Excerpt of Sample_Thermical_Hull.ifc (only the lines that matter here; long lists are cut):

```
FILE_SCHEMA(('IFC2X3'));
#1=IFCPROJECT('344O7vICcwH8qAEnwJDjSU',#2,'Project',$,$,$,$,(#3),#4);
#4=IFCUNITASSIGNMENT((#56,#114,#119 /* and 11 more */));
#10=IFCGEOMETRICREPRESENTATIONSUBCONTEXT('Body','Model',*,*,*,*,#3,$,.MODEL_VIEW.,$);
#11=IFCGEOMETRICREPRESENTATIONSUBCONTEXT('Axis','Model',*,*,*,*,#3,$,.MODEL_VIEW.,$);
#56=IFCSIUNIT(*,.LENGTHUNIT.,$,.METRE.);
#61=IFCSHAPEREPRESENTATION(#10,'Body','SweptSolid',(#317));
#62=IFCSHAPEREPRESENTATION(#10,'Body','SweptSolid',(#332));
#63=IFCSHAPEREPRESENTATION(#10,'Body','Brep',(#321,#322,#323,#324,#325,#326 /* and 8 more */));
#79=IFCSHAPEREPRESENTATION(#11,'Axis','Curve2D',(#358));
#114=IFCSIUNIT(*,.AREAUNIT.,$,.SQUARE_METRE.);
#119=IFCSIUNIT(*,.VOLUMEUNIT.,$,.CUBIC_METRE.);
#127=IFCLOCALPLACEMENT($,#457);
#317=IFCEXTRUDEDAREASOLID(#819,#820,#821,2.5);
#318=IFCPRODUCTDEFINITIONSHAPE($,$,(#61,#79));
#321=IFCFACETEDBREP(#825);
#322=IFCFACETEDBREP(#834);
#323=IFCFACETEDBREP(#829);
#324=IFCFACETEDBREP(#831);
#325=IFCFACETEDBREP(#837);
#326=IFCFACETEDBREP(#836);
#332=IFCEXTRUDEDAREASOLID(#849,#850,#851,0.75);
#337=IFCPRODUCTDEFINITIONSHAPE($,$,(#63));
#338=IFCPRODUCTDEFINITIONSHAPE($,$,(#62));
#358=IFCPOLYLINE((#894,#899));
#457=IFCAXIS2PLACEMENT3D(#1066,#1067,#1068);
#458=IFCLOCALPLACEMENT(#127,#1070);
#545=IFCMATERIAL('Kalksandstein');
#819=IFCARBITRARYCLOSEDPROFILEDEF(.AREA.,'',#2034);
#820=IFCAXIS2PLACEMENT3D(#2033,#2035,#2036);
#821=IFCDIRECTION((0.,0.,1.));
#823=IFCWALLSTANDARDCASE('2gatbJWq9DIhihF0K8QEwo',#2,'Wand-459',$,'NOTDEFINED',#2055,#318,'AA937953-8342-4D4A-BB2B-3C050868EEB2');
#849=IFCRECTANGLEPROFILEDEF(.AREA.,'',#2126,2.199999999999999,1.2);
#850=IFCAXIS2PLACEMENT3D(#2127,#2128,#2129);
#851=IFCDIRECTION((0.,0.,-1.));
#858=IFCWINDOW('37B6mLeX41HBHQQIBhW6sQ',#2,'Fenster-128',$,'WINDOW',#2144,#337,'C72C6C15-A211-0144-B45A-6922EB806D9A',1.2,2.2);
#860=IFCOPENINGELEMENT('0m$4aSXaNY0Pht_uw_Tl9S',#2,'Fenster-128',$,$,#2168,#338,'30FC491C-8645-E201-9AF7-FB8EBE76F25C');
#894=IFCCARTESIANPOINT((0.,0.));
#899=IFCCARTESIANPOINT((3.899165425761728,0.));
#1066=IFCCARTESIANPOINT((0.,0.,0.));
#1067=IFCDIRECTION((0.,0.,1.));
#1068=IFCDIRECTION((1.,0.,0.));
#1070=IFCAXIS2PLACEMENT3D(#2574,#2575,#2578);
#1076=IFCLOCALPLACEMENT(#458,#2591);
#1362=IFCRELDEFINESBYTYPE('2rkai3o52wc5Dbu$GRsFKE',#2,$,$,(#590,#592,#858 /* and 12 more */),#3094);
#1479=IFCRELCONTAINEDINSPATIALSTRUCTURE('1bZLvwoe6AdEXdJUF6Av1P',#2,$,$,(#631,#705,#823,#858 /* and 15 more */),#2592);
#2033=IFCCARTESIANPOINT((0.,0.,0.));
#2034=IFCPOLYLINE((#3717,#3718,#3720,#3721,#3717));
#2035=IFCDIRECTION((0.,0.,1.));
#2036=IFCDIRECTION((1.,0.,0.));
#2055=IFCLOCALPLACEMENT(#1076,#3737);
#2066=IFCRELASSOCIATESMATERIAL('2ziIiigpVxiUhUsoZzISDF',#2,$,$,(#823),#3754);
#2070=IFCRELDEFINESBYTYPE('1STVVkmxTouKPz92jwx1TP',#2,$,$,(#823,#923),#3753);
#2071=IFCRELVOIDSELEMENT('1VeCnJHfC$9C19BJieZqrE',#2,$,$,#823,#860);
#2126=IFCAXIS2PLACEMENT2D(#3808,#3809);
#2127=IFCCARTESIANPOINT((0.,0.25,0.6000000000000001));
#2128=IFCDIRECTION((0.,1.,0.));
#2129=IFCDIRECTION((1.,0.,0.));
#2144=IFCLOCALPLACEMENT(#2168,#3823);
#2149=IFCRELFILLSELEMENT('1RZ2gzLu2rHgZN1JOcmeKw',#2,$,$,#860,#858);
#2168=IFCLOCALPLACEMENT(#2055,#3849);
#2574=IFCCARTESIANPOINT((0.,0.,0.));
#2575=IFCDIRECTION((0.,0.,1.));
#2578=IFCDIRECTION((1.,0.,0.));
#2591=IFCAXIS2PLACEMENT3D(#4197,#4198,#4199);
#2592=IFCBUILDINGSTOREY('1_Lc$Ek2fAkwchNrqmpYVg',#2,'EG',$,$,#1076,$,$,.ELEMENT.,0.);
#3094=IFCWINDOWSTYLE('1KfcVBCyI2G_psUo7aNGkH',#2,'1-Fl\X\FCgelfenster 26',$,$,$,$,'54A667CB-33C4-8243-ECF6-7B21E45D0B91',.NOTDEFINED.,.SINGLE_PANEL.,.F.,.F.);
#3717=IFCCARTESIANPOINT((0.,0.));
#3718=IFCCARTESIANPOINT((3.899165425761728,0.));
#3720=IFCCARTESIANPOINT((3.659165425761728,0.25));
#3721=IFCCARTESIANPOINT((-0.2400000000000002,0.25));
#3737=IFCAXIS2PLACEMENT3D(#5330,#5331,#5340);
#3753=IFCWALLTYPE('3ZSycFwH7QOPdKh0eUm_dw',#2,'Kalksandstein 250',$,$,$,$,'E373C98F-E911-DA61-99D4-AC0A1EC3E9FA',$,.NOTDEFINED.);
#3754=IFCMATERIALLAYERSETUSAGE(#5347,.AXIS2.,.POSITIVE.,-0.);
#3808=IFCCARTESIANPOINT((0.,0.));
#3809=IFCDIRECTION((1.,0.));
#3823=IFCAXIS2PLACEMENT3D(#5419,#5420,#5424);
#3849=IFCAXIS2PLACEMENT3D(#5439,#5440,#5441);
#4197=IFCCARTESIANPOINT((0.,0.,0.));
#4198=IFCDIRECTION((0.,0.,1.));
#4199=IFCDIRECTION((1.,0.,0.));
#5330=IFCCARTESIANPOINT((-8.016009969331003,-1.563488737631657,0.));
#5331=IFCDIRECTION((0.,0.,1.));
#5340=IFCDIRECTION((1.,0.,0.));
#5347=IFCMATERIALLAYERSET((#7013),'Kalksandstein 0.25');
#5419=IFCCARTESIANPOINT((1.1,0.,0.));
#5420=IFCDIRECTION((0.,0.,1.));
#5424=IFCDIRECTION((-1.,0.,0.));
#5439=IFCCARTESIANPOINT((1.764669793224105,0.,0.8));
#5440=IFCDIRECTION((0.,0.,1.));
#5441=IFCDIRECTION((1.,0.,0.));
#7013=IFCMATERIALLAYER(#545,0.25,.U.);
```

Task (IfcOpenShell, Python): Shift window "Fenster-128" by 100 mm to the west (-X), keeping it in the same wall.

```python
import ifcopenshell
import ifcopenshell.api.geometry
import ifcopenshell.util.placement
import ifcopenshell.util.unit

model = ifcopenshell.open("Sample_Thermical_Hull.ifc")
unit_scale = ifcopenshell.util.unit.calculate_unit_scale(model)

window = model.by_id(858)
opening = window.FillsVoids[0].RelatingOpeningElement
wall = opening.VoidsElements[0].RelatingBuildingElement

wall_matrix = ifcopenshell.util.placement.get_local_placement(wall.ObjectPlacement)
shift = wall_matrix[:3, 0] * -0.1 / unit_scale
before = ifcopenshell.util.placement.get_local_placement(window.ObjectPlacement)[:3, 3].copy()

# The window is placed relative to its opening, so it follows when the opening moves.
matrix = ifcopenshell.util.placement.get_local_placement(opening.ObjectPlacement)
matrix[:3, 3] += shift
ifcopenshell.api.geometry.edit_object_placement(
    model, product=opening, matrix=matrix, is_si=False, should_transform_children=True
)

after = ifcopenshell.util.placement.get_local_placement(window.ObjectPlacement)[:3, 3]
print("window moved by", (after - before).round(3) + 0.0)

model.write("Sample_Thermical_Hull_v2.ifc")
```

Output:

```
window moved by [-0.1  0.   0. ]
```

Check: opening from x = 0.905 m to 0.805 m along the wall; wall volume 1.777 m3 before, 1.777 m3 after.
